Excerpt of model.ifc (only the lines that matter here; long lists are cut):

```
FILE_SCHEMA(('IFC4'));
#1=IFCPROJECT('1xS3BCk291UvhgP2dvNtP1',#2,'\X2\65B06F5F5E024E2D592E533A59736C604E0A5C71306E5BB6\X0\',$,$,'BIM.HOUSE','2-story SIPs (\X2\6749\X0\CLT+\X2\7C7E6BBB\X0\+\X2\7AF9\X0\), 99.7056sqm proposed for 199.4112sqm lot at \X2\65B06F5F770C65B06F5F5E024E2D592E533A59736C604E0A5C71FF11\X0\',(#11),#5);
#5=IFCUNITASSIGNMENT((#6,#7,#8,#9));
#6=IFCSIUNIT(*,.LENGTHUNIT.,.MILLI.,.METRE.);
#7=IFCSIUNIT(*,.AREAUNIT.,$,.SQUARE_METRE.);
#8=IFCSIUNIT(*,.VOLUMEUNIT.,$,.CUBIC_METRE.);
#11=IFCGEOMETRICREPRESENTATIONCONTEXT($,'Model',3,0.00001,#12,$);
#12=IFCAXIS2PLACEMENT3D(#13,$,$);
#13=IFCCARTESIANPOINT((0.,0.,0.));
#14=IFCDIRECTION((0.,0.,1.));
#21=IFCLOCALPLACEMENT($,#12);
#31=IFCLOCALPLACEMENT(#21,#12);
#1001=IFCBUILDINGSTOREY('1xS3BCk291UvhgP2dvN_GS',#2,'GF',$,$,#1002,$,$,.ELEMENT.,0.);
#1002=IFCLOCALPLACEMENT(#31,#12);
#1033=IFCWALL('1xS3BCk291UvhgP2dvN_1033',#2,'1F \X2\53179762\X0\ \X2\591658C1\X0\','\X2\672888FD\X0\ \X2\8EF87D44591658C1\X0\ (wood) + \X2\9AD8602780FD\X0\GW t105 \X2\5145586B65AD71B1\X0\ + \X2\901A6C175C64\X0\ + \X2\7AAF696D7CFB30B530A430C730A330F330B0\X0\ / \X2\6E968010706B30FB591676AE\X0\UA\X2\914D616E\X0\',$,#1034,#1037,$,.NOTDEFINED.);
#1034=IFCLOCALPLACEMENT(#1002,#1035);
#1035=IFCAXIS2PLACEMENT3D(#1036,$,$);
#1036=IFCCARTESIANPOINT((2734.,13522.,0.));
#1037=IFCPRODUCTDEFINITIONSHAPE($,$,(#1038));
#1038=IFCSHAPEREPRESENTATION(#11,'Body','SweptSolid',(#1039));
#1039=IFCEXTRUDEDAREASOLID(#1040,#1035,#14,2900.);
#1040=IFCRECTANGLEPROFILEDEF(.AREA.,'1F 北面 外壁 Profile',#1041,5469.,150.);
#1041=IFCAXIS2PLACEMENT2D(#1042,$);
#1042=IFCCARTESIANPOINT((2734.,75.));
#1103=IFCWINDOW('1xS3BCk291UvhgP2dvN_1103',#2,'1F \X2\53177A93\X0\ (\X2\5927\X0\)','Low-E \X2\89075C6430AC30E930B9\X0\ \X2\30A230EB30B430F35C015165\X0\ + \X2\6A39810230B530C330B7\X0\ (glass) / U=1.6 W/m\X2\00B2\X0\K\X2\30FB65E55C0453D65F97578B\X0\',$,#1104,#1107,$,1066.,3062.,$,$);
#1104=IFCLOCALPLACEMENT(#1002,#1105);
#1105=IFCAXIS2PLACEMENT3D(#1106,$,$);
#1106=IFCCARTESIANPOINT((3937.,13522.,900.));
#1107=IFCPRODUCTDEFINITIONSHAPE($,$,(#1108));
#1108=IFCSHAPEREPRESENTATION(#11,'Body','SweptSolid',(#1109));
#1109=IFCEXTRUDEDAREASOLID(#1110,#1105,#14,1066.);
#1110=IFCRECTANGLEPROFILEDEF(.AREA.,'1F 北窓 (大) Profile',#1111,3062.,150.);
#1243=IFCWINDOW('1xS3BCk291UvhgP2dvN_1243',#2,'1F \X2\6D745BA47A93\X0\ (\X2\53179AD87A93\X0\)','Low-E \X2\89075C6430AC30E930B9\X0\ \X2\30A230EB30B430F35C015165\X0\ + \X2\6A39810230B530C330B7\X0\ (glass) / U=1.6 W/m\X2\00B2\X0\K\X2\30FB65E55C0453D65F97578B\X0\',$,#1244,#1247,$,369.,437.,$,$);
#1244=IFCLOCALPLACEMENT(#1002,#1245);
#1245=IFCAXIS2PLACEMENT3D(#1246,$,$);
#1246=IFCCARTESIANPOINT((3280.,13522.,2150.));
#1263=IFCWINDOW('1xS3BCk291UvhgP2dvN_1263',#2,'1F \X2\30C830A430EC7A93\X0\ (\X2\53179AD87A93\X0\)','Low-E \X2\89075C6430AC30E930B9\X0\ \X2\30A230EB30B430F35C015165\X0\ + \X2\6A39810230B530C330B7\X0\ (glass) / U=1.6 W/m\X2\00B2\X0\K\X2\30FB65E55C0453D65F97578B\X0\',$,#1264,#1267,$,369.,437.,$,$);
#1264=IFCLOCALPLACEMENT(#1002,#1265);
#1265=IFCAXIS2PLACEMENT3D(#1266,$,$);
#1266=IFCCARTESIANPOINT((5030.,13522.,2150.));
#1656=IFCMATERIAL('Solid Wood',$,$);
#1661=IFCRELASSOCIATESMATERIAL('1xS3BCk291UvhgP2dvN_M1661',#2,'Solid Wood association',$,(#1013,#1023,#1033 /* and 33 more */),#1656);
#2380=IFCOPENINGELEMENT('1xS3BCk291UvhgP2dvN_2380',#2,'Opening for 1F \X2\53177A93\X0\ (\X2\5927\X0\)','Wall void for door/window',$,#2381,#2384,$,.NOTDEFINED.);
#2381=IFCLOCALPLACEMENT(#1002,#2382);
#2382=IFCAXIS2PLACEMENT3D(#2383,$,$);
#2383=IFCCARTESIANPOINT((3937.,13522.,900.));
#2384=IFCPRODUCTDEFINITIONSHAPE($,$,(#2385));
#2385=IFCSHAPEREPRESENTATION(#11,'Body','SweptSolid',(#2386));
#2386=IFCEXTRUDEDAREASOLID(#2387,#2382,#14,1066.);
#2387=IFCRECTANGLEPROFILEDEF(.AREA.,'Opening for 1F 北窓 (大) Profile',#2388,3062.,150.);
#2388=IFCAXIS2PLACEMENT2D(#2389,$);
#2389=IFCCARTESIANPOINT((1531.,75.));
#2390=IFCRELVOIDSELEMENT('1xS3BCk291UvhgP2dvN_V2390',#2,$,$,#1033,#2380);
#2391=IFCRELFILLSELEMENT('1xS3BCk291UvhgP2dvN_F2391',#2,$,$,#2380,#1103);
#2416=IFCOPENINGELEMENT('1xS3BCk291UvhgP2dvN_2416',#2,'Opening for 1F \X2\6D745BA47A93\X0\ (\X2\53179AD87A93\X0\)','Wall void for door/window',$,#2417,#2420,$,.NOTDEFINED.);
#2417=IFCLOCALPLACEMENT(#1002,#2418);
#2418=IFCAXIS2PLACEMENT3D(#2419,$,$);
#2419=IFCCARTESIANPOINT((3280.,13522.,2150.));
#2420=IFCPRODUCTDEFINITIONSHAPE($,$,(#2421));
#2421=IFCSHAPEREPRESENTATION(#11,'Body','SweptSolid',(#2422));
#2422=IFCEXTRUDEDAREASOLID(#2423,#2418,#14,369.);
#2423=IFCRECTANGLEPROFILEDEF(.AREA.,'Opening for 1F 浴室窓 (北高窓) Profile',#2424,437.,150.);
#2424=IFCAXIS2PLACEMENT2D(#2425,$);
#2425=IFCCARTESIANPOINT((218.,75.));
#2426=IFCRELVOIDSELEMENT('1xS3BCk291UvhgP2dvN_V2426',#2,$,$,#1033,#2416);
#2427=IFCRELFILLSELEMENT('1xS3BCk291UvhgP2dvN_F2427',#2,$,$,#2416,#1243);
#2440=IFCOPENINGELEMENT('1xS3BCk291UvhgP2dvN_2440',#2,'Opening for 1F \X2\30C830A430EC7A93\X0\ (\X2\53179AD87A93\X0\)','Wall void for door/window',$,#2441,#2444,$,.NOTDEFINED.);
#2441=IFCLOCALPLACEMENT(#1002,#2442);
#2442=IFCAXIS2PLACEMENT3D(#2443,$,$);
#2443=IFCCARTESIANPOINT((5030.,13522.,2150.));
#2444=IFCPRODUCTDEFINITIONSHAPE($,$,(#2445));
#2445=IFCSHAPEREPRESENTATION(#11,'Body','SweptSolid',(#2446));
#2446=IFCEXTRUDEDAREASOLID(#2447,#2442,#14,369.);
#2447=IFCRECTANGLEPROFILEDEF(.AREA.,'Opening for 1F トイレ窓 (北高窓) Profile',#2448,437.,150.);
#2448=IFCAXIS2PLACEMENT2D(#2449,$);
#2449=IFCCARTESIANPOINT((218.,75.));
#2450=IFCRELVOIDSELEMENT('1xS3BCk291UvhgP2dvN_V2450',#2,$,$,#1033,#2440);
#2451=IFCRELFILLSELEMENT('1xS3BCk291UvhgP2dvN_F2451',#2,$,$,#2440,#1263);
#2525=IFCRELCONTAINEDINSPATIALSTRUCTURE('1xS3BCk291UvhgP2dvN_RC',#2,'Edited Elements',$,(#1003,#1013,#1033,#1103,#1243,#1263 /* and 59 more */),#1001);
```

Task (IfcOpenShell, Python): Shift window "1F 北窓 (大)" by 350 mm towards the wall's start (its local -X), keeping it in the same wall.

```python
import ifcopenshell
import ifcopenshell.api.geometry
import ifcopenshell.util.placement
import ifcopenshell.util.unit

model = ifcopenshell.open("model.ifc")
unit_scale = ifcopenshell.util.unit.calculate_unit_scale(model)

window = model.by_guid("1xS3BCk291UvhgP2dvN_1103")
opening = window.FillsVoids[0].RelatingOpeningElement
wall = opening.VoidsElements[0].RelatingBuildingElement

wall_matrix = ifcopenshell.util.placement.get_local_placement(wall.ObjectPlacement)
shift = wall_matrix[:3, 0] * -0.35 / unit_scale
before = ifcopenshell.util.placement.get_local_placement(window.ObjectPlacement)[:3, 3].copy()

# The window is not placed relative to its opening, so move both.
for product in (opening, window):
    matrix = ifcopenshell.util.placement.get_local_placement(product.ObjectPlacement)
    matrix[:3, 3] += shift
    ifcopenshell.api.geometry.edit_object_placement(model, product=product, matrix=matrix, is_si=False)

after = ifcopenshell.util.placement.get_local_placement(window.ObjectPlacement)[:3, 3]
print("window moved by", (after - before).round(3) + 0.0)

model.write("model_v2.ifc")
```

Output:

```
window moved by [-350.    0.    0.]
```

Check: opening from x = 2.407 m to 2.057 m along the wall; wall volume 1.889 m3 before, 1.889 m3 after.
